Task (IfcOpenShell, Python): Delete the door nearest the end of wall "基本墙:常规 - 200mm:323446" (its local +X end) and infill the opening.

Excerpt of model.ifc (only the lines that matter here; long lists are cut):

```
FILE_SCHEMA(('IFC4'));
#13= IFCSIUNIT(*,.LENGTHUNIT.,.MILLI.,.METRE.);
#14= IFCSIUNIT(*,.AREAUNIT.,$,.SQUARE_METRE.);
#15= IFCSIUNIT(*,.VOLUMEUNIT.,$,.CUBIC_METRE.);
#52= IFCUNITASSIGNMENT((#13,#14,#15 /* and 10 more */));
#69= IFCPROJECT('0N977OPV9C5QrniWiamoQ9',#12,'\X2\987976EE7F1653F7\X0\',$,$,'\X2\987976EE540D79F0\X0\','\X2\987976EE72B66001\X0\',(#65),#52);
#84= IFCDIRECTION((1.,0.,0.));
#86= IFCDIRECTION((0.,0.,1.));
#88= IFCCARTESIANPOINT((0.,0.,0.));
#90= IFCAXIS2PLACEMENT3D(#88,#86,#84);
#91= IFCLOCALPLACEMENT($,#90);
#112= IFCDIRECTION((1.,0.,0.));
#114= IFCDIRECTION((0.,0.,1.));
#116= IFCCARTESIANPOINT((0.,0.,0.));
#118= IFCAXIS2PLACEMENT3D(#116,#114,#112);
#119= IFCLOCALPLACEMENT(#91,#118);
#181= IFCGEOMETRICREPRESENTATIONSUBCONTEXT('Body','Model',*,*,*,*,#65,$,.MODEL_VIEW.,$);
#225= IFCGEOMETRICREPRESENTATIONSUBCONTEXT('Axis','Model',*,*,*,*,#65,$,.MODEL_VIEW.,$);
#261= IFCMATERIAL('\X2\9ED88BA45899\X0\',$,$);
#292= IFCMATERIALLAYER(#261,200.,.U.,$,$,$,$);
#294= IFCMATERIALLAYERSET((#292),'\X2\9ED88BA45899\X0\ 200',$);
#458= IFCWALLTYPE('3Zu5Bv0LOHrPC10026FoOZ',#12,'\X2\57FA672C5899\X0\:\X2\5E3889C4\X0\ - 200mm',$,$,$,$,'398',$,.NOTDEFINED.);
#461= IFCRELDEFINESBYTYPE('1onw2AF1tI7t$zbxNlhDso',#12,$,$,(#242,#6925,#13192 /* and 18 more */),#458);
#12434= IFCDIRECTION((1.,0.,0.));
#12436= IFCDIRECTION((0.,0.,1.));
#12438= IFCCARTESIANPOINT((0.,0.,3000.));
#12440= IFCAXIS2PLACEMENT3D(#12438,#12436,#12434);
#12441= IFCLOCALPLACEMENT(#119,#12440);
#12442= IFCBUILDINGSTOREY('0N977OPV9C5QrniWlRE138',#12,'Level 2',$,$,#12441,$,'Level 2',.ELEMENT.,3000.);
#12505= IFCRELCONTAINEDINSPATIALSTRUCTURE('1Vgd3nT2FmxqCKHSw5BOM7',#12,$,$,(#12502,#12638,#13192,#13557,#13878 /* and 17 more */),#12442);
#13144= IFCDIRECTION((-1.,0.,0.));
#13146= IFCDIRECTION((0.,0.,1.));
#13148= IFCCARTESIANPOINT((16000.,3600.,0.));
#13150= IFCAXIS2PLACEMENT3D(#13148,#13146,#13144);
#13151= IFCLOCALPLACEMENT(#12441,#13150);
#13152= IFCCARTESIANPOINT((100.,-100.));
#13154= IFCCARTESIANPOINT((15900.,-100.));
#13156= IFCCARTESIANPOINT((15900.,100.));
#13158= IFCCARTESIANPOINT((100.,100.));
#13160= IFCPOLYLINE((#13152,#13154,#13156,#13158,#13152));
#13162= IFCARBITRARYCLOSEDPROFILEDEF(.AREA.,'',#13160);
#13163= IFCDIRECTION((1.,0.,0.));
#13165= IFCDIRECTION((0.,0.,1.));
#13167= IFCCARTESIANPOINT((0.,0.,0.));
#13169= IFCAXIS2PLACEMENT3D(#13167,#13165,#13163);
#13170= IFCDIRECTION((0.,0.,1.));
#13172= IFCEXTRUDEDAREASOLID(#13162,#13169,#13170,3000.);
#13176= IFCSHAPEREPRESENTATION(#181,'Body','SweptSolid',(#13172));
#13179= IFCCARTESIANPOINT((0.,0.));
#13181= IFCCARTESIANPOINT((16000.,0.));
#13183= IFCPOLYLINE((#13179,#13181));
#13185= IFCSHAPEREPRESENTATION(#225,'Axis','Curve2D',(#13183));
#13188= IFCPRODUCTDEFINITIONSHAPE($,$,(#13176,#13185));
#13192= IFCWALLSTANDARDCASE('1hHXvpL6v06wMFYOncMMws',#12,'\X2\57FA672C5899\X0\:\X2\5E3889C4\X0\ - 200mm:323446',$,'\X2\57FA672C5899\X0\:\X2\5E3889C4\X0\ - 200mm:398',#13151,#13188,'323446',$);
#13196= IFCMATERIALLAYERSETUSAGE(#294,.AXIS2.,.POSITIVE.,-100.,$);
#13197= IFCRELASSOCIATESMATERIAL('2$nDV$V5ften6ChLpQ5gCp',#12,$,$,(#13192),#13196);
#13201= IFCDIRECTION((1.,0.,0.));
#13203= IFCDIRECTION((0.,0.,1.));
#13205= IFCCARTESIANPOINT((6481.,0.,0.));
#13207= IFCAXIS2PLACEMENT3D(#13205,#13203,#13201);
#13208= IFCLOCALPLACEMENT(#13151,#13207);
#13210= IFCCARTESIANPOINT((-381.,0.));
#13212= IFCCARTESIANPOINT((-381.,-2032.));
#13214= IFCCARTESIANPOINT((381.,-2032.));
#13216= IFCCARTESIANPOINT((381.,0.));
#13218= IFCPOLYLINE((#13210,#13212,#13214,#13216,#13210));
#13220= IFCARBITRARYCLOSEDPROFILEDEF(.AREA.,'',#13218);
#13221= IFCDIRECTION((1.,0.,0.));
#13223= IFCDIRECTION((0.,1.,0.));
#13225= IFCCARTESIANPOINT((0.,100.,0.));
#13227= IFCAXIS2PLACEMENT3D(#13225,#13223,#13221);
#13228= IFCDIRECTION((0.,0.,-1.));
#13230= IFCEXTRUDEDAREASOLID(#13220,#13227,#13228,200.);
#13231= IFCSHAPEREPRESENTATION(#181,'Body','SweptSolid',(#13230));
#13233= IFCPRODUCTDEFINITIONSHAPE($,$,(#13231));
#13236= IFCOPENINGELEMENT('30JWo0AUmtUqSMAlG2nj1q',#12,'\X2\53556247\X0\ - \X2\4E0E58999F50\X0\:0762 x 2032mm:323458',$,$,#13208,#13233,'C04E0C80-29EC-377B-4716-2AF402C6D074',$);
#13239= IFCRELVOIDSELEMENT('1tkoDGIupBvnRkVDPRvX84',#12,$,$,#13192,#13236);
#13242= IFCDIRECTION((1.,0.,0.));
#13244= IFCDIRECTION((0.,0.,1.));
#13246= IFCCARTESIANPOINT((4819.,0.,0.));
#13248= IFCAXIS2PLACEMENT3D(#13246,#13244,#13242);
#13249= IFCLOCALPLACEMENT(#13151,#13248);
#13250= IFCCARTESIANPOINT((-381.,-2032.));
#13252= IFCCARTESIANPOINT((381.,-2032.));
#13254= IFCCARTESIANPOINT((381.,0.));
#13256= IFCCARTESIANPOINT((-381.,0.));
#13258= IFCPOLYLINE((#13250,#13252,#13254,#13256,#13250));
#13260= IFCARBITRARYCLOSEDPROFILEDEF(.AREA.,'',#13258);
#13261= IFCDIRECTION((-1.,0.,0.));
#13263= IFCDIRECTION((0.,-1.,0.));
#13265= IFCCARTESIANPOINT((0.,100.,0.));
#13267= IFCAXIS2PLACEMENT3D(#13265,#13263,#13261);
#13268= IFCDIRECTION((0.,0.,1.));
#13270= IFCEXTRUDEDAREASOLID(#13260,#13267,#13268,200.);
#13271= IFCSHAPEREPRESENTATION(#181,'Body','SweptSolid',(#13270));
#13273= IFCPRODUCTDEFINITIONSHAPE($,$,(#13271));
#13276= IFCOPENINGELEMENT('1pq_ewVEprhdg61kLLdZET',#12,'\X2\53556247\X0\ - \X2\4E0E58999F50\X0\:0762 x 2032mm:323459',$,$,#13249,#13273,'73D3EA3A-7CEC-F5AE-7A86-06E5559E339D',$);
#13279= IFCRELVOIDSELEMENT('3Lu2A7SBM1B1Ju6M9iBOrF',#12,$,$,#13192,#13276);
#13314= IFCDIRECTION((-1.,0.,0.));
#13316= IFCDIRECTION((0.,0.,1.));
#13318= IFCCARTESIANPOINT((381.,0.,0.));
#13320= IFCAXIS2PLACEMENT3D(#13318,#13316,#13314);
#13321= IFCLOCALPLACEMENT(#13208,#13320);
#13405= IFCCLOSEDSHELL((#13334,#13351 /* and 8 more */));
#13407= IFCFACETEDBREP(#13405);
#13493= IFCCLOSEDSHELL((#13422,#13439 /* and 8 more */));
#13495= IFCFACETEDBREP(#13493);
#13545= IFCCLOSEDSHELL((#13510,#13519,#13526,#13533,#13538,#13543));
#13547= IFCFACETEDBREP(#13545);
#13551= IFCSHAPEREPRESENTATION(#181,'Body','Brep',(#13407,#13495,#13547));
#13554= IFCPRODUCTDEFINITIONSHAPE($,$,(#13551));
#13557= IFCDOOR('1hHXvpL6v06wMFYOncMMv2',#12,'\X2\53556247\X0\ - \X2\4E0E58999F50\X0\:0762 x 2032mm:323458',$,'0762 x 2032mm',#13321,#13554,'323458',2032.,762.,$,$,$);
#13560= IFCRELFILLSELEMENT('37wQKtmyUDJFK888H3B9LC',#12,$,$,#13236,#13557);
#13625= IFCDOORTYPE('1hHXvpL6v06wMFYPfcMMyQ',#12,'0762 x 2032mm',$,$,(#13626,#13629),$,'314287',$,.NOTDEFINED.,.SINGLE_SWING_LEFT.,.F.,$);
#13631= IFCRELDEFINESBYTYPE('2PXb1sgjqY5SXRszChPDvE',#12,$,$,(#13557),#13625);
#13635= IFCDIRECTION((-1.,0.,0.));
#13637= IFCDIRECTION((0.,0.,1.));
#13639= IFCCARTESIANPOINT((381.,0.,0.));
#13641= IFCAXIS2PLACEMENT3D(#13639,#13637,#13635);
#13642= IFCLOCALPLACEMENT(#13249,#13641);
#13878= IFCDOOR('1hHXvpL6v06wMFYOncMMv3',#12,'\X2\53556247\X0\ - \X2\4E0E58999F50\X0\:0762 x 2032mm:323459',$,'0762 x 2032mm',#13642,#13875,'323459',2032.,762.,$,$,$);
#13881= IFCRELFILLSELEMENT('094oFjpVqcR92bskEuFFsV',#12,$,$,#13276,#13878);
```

```python
import ifcopenshell
import ifcopenshell.api.feature
import ifcopenshell.api.root
import ifcopenshell.geom
import ifcopenshell.util.shape

model = ifcopenshell.open("model.ifc")
settings = ifcopenshell.geom.settings()


def volume(element):
    """Net volume in cubic metres, openings subtracted."""
    shape = ifcopenshell.geom.create_shape(settings, element)
    return ifcopenshell.util.shape.get_volume(shape.geometry)


door = model.by_guid("1hHXvpL6v06wMFYOncMMv2")
opening = door.FillsVoids[0].RelatingOpeningElement
wall = opening.VoidsElements[0].RelatingBuildingElement
before = volume(wall)

ifcopenshell.api.root.remove_product(model, product=door)
ifcopenshell.api.feature.remove_feature(model, feature=opening)

after = volume(wall)

print(f"wall volume {before:.3f} -> {after:.3f} m3")

model.write("model-out.ifc")
```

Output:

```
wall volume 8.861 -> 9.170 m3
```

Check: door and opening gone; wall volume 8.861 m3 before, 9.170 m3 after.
